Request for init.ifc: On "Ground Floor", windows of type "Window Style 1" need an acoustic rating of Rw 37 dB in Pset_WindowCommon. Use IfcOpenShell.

First a look at what the model holds.

```python
import ifcopenshell
import ifcopenshell.util.element

model = ifcopenshell.open("init.ifc")
print(model.schema)
storey = next(s for s in model.by_type("IfcBuildingStorey") if s.Name == "Ground Floor")
windows = [e for e in ifcopenshell.util.element.get_decomposition(storey) if e.is_a("IfcWindow")]
seen = {}
for e in windows:
    element_type = ifcopenshell.util.element.get_type(e)
    key = (element_type.Name if element_type != e and element_type else None, ifcopenshell.util.element.get_pset(e, "Pset_WindowCommon", "AcousticRating"))
    seen[key] = seen.get(key, 0) + 1
for (name, value), count in sorted(seen.items(), key=str):
    print(count, "x", name, "|", value)
```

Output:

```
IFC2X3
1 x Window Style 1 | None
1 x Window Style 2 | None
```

```python
import ifcopenshell
import ifcopenshell.api.pset
import ifcopenshell.util.element

model = ifcopenshell.open("init.ifc")

storey = next(s for s in model.by_type("IfcBuildingStorey") if s.Name == "Ground Floor")
windows = [e for e in ifcopenshell.util.element.get_decomposition(storey) if e.is_a("IfcWindow")]

count = 0
for e in windows:
    element_type = ifcopenshell.util.element.get_type(e)
    if element_type in (None, e) or element_type.Name != "Window Style 1":
        continue
    # add_pset returns the element's existing set when there is one.
    pset = ifcopenshell.api.pset.add_pset(model, product=e, name="Pset_WindowCommon")
    ifcopenshell.api.pset.edit_pset(model, pset=pset, properties={"AcousticRating": "Rw 37 dB"})
    count += 1

print(count, "windows updated")

model.write("init_updated.ifc")
```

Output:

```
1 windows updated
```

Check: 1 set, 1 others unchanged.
